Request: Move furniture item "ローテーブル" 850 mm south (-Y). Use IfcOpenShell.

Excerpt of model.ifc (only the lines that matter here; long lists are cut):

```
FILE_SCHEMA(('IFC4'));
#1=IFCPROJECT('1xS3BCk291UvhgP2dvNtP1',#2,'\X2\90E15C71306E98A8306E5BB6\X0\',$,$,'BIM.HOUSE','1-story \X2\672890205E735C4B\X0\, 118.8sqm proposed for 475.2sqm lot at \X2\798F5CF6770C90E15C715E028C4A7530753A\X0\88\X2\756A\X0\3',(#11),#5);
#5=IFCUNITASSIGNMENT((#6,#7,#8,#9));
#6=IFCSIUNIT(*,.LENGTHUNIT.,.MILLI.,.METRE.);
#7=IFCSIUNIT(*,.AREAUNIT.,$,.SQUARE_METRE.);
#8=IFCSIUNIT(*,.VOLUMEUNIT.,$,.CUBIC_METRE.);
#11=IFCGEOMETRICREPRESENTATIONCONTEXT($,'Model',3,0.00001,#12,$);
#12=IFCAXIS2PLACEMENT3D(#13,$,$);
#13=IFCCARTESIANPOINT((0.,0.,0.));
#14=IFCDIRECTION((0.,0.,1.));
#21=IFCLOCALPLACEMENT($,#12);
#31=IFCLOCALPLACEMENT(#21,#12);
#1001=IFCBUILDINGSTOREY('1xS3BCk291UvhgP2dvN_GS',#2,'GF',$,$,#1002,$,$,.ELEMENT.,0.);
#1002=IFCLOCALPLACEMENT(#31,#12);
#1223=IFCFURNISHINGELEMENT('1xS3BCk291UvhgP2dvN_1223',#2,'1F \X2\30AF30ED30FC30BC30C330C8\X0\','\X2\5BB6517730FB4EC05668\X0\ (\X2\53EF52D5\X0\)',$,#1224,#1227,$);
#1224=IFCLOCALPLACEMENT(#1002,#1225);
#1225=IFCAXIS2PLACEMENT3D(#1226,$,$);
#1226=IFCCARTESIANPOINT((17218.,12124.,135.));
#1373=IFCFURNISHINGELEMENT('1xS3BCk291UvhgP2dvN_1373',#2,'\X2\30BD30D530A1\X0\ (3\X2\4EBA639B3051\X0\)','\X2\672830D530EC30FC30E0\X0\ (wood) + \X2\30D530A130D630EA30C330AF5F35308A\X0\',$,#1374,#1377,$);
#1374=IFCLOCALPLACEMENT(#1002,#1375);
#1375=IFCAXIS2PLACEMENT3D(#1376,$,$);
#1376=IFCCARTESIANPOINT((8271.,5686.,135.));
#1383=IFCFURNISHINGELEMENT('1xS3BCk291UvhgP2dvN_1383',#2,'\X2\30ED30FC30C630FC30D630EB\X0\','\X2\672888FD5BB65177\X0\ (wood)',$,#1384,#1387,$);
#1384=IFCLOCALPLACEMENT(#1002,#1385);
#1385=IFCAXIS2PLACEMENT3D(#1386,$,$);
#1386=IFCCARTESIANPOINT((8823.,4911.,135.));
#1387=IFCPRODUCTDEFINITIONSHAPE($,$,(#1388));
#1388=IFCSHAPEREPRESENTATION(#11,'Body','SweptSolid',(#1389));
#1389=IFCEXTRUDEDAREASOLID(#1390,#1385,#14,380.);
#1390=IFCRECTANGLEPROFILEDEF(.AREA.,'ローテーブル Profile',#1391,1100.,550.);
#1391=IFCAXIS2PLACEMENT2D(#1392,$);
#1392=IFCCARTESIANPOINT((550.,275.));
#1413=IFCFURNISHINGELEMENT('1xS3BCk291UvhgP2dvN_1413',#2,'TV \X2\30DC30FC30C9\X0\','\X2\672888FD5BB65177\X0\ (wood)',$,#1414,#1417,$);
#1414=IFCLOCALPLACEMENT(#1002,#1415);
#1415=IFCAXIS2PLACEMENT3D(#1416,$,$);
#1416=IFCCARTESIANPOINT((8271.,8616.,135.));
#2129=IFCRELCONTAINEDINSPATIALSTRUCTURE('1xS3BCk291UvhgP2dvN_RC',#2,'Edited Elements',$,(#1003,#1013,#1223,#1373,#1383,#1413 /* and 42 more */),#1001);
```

```python
import ifcopenshell
import ifcopenshell.api.geometry
import ifcopenshell.util.placement

model = ifcopenshell.open("model.ifc")

item = model.by_guid("1xS3BCk291UvhgP2dvN_1383")
matrix = ifcopenshell.util.placement.get_local_placement(item.ObjectPlacement)
matrix[1, 3] -= 850.0
ifcopenshell.api.geometry.edit_object_placement(model, product=item, matrix=matrix, is_si=False)

print(ifcopenshell.util.placement.get_local_placement(item.ObjectPlacement).round(3) + 0.0)

model.write("model-out.ifc")
```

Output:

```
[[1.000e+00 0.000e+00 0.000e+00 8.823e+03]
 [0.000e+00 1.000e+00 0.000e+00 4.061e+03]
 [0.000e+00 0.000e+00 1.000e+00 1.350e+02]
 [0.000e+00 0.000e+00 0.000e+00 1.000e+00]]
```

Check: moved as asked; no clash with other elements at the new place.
